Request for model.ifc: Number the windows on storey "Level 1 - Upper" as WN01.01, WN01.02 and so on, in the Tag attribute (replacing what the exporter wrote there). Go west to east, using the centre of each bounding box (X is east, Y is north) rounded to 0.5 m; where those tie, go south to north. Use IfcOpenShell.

First a look at what the model holds.

```python
import ifcopenshell
import ifcopenshell.util.element
import ifcopenshell.util.placement

model = ifcopenshell.open("model.ifc")
print(model.schema)
storey = next(s for s in model.by_type("IfcBuildingStorey") if s.Name == "Level 1 - Upper")
windows = [e for e in ifcopenshell.util.element.get_decomposition(storey) if e.is_a("IfcWindow")]
for e in sorted(windows, key=lambda e: e.id()):
    origin = ifcopenshell.util.placement.get_local_placement(e.ObjectPlacement)[:3, 3]
    print(e.id(), e.Tag, e.Name, origin.round(2) + 0.0, sep=" | ")
```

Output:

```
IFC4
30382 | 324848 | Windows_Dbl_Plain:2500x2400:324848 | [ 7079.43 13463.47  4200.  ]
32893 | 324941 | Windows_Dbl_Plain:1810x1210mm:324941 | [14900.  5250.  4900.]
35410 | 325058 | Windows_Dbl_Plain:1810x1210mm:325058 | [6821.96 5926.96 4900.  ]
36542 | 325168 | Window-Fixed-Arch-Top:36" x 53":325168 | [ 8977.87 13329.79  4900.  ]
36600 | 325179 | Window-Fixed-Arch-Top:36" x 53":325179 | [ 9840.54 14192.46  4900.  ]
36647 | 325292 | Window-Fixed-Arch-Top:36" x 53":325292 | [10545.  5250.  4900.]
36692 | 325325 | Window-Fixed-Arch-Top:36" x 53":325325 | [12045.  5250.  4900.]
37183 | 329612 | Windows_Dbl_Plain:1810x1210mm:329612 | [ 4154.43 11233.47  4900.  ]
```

```python
import ifcopenshell
import ifcopenshell.geom
import ifcopenshell.util.element
import ifcopenshell.util.shape

model = ifcopenshell.open("model.ifc")
settings = ifcopenshell.geom.settings()
settings.set("use-world-coords", True)


def centre(element):
    shape = ifcopenshell.geom.create_shape(settings, element)
    return ifcopenshell.util.shape.get_bbox_centroid(shape.geometry)


storey = next(s for s in model.by_type("IfcBuildingStorey") if s.Name == "Level 1 - Upper")
windows = [e for e in ifcopenshell.util.element.get_decomposition(storey) if e.is_a("IfcWindow")]

# Insertion points can sit at a corner or the storey origin, so sort by the geometry (in metres).
centres = {e: centre(e) for e in windows}
windows.sort(key=lambda e: (round(centres[e][0] / 0.5), centres[e][1]))

for i, e in enumerate(windows, start=1):
    number = f"WN01.{i:02d}"
    e.Tag = number
    print(e.id(), number)

model.write("model_edited.ifc")
```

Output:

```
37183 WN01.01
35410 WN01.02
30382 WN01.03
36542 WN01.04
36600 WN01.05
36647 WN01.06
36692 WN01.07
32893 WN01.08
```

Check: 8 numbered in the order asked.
